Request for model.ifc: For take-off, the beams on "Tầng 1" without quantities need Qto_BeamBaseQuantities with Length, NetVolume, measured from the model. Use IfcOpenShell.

First a look at what the model holds.

```python
import ifcopenshell
import ifcopenshell.util.element
import ifcopenshell.util.unit

model = ifcopenshell.open("model.ifc")
print(model.schema)
for unit_type in ("LENGTHUNIT", "AREAUNIT", "VOLUMEUNIT"):
    print(unit_type, ifcopenshell.util.unit.calculate_unit_scale(model, unit_type))
storey = next(s for s in model.by_type("IfcBuildingStorey") if s.Name == "Tầng 1")
beams = [e for e in ifcopenshell.util.element.get_decomposition(storey) if e.is_a("IfcBeam")]
for e in sorted(beams, key=lambda e: e.id()):
    print(e.id(), e.is_a(), e.Name, list(ifcopenshell.util.element.get_psets(e, qtos_only=True)), sep=" | ")
```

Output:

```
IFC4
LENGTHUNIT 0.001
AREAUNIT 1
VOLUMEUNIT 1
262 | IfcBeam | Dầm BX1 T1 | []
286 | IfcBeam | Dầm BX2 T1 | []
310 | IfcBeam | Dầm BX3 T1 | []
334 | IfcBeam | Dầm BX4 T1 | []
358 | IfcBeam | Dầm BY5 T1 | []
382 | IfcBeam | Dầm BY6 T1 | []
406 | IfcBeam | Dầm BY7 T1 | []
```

```python
import ifcopenshell
import ifcopenshell.api.pset
import ifcopenshell.geom
import ifcopenshell.util.element
import ifcopenshell.util.shape
import ifcopenshell.util.unit

model = ifcopenshell.open("model.ifc")
unit_scale = ifcopenshell.util.unit.calculate_unit_scale(model)
volume_scale = ifcopenshell.util.unit.calculate_unit_scale(model, "VOLUMEUNIT")
settings = ifcopenshell.geom.settings()

storey = next(s for s in model.by_type("IfcBuildingStorey") if s.Name == "Tầng 1")
beams = [e for e in ifcopenshell.util.element.get_decomposition(storey) if e.is_a("IfcBeam")]

for e in sorted(beams, key=lambda e: e.id()):
    if ifcopenshell.util.element.get_psets(e, qtos_only=True, should_inherit=False):
        continue
    # Geometry comes back in metres, in the element's own axes.
    shape = ifcopenshell.geom.create_shape(settings, e)
    values = {
        "Length": ifcopenshell.util.shape.get_max_xyz(shape.geometry) / unit_scale,
        "NetVolume": ifcopenshell.util.shape.get_volume(shape.geometry) / volume_scale,
    }
    qto = ifcopenshell.api.pset.add_qto(model, product=e, name="Qto_BeamBaseQuantities")
    ifcopenshell.api.pset.edit_qto(model, qto=qto, properties=values)
    print(e.id(), {k: round(v, 3) for k, v in values.items()})

model.write("model_updated.ifc")
```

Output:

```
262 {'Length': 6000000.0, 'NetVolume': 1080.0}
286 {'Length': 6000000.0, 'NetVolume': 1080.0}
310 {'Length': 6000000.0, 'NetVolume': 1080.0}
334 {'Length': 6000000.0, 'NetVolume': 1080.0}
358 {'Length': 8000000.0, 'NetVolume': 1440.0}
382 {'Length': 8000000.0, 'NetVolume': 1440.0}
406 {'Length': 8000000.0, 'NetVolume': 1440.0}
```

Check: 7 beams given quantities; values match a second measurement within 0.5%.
